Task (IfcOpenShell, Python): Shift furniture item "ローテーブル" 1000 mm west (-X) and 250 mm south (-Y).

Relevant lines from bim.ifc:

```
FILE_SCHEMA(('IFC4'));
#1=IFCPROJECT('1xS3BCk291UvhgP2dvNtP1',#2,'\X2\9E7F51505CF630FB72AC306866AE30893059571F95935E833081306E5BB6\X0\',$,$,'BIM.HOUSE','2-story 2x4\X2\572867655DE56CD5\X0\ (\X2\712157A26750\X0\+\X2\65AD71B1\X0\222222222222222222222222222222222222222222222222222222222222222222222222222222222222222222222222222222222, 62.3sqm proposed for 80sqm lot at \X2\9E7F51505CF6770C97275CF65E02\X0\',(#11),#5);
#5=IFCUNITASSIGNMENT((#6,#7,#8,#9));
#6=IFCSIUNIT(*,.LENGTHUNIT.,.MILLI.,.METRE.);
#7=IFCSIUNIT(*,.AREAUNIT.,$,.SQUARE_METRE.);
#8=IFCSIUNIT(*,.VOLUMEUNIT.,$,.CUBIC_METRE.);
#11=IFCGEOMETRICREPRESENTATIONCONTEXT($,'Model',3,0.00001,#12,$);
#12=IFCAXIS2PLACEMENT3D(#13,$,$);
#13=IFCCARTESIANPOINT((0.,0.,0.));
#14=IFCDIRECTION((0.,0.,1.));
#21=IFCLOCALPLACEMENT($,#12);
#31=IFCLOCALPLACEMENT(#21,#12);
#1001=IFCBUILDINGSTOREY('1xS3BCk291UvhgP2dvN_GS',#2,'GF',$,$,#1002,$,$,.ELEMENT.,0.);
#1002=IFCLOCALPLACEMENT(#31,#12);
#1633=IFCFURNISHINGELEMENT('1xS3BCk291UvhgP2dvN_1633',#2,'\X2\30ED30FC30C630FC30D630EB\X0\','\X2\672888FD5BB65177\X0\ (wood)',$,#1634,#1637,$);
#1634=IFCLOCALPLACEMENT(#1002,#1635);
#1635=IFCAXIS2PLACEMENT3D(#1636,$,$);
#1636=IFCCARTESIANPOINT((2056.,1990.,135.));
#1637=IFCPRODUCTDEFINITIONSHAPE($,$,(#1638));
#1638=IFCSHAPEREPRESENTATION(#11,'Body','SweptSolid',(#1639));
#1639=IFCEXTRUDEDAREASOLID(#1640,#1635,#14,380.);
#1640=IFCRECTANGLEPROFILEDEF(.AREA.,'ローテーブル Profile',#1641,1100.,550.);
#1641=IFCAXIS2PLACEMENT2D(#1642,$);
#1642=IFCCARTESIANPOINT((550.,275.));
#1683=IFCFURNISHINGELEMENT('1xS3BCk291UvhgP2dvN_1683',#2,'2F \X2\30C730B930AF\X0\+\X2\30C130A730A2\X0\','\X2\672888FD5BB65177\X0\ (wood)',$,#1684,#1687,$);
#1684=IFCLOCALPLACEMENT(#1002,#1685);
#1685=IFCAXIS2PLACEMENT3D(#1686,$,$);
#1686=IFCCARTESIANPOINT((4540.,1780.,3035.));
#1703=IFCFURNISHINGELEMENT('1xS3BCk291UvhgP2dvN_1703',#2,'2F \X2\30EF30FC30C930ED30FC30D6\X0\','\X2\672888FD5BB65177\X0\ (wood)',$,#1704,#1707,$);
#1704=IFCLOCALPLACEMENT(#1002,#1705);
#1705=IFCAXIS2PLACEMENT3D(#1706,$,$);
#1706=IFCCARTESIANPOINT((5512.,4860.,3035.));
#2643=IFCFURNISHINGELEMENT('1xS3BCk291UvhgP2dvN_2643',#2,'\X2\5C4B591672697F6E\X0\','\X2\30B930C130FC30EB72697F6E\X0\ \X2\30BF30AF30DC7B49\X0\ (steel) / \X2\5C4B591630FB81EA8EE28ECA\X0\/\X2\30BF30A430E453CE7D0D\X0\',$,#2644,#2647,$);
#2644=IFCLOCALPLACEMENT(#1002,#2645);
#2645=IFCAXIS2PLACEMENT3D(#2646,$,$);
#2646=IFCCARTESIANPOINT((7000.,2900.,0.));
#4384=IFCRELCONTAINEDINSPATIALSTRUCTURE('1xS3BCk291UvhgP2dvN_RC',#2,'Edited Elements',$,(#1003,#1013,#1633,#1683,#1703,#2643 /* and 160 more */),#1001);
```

```python
import ifcopenshell
import ifcopenshell.api.geometry
import ifcopenshell.util.placement

model = ifcopenshell.open("bim.ifc")

item = model.by_id(1633)
matrix = ifcopenshell.util.placement.get_local_placement(item.ObjectPlacement)
matrix[0, 3] -= 1000.0
matrix[1, 3] -= 250.0
ifcopenshell.api.geometry.edit_object_placement(model, product=item, matrix=matrix, is_si=False)

print(ifcopenshell.util.placement.get_local_placement(item.ObjectPlacement).round(3) + 0.0)

model.write("bim_updated.ifc")
```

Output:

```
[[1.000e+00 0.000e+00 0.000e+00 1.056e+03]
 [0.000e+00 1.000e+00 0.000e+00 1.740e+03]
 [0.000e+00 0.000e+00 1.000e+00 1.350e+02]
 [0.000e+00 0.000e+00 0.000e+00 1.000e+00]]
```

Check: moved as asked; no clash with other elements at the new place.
